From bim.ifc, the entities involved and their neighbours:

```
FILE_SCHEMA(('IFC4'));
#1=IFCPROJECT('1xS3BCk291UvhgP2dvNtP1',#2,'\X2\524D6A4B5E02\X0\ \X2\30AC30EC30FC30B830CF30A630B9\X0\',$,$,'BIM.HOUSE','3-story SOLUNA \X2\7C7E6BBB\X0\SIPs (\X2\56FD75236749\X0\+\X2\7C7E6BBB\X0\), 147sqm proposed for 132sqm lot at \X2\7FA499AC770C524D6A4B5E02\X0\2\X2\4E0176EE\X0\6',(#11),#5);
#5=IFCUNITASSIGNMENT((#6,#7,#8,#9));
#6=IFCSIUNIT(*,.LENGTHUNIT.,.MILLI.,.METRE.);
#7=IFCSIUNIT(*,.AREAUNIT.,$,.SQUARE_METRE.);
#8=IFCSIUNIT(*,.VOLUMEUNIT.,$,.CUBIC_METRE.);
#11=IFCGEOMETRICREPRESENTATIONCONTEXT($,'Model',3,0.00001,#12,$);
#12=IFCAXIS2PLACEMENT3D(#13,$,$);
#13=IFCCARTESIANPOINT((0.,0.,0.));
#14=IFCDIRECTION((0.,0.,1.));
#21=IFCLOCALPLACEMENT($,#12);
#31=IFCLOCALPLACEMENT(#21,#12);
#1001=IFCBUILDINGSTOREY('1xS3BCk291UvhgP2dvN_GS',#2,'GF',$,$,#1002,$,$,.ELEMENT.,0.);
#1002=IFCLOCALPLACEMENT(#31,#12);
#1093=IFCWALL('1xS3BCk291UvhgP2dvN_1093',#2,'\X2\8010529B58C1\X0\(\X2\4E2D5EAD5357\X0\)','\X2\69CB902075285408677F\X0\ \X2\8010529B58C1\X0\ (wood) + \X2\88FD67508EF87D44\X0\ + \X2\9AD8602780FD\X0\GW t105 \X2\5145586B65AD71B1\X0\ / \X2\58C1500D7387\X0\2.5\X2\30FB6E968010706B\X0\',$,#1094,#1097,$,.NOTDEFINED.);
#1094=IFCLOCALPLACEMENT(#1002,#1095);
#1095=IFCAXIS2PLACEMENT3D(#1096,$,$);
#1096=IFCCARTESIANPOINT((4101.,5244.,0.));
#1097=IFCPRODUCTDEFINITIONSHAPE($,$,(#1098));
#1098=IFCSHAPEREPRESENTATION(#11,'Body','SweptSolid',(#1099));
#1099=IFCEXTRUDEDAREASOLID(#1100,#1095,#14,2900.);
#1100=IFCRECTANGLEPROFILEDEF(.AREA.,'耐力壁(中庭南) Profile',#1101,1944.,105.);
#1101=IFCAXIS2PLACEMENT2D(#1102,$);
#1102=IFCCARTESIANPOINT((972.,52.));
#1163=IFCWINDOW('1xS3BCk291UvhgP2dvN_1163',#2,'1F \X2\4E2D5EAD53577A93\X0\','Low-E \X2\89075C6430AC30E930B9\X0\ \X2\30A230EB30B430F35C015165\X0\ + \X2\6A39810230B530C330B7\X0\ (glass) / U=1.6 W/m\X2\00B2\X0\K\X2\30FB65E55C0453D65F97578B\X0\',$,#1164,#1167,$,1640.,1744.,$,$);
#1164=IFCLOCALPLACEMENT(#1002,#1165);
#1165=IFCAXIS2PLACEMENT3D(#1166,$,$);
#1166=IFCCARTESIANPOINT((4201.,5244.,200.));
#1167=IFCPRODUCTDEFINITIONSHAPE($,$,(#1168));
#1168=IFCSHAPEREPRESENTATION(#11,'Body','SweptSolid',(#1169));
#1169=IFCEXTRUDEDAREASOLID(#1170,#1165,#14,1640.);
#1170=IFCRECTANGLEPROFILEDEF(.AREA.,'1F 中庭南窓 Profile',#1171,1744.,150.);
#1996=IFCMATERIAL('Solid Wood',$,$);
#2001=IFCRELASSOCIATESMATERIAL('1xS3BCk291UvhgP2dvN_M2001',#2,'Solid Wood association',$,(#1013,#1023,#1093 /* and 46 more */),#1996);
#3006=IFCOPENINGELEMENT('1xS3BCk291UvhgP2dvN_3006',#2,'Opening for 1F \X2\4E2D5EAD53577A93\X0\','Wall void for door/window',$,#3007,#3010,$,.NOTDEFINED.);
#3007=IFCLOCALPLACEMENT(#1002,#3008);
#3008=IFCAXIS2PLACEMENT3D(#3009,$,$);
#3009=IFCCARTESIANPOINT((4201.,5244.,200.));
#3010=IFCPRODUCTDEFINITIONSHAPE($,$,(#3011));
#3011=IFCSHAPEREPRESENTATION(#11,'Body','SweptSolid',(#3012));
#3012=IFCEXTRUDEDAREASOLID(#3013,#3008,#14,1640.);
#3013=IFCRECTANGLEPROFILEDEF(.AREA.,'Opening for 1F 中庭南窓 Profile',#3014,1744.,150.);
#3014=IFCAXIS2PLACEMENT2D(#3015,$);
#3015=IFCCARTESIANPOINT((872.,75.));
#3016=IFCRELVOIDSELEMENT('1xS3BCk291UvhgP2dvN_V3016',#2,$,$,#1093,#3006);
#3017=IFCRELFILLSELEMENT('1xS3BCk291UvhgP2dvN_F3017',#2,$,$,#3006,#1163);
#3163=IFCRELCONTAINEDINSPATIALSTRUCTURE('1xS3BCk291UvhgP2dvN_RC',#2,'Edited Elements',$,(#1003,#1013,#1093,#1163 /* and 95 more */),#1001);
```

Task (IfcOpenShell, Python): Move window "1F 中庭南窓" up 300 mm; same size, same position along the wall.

```python
import numpy as np
import ifcopenshell
import ifcopenshell.api.geometry
import ifcopenshell.util.placement
import ifcopenshell.util.unit

model = ifcopenshell.open("bim.ifc")
unit_scale = ifcopenshell.util.unit.calculate_unit_scale(model)

window = model.by_guid("1xS3BCk291UvhgP2dvN_1163")
opening = window.FillsVoids[0].RelatingOpeningElement
dz = 0.3 / unit_scale

shift = np.array([0.0, 0.0, dz])
# The window is not placed relative to its opening, so move both.
for product in (opening, window):
    matrix = ifcopenshell.util.placement.get_local_placement(product.ObjectPlacement)
    matrix[:3, 3] += shift
    ifcopenshell.api.geometry.edit_object_placement(model, product=product, matrix=matrix, is_si=False)

print(f"moved by {dz * unit_scale:+.3f} m")

model.write("bim_edited.ifc")
```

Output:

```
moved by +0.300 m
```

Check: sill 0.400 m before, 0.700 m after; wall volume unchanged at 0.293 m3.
